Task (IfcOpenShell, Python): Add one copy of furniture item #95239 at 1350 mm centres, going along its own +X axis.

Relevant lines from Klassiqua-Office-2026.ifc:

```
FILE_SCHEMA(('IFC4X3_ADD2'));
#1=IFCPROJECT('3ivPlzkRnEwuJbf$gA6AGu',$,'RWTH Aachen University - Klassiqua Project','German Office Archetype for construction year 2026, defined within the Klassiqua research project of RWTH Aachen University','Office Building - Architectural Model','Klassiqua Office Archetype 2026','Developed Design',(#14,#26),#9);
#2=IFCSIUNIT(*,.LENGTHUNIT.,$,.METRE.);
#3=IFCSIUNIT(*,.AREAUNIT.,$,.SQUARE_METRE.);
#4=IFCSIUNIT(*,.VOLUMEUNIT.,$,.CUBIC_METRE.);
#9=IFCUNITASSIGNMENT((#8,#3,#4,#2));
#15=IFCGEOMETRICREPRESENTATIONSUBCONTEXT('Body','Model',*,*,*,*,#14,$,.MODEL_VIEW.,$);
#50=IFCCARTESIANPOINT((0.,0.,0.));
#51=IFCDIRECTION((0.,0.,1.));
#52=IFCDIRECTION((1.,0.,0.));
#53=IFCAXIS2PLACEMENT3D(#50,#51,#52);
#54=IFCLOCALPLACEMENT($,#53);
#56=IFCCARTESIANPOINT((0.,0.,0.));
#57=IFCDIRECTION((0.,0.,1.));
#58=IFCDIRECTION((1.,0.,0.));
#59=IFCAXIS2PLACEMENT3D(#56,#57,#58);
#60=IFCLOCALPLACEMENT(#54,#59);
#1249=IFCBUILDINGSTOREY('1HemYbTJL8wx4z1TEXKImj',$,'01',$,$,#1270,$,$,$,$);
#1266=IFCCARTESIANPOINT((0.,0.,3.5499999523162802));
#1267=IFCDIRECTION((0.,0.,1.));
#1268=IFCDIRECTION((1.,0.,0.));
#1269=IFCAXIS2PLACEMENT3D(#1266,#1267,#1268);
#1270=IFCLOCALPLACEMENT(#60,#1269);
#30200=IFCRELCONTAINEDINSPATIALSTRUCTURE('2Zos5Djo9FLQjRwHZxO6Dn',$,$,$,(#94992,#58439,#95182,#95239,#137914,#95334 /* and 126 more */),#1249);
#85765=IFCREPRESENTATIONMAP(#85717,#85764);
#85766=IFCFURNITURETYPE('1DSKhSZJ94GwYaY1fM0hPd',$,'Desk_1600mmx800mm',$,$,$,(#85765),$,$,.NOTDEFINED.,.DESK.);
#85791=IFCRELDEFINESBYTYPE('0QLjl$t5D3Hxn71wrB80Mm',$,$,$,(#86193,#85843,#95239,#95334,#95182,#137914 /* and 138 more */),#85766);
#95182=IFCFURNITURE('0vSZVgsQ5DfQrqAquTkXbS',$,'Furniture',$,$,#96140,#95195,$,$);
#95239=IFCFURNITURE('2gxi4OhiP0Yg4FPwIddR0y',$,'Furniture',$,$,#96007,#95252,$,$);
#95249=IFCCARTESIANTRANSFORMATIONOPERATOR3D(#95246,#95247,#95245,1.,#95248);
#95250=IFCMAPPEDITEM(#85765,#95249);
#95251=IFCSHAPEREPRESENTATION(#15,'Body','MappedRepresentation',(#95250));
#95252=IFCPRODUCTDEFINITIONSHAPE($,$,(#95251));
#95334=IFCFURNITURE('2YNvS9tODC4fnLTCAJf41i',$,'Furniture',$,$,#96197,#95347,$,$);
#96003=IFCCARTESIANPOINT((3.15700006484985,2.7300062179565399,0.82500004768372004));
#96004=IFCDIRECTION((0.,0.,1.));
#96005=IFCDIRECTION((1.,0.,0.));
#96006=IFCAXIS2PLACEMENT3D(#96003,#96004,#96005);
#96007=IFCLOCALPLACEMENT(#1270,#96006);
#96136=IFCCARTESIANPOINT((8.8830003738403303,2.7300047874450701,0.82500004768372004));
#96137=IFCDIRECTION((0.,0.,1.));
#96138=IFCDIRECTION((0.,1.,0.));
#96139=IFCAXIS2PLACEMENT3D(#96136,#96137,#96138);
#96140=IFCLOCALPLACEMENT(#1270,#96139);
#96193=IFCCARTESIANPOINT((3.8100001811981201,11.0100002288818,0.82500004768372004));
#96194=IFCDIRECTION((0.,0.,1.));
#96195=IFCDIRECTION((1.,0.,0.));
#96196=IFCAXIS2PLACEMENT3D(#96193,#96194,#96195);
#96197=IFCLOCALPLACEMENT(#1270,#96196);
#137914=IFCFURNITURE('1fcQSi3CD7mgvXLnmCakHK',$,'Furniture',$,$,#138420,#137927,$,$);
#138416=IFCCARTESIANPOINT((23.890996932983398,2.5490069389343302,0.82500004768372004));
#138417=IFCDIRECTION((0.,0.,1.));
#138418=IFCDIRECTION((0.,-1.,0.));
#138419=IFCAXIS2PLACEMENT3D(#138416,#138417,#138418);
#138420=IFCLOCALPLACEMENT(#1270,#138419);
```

```python
import ifcopenshell
import ifcopenshell.api.geometry
import ifcopenshell.api.root
import ifcopenshell.util.element
import ifcopenshell.util.placement

model = ifcopenshell.open("Klassiqua-Office-2026.ifc")

source = model.by_guid("2gxi4OhiP0Yg4FPwIddR0y")
base = ifcopenshell.util.placement.get_local_placement(source.ObjectPlacement)
step = base[:3, 0] * 1.35

for i in range(1, 2):
    copy = ifcopenshell.api.root.copy_class(model, product=source)
    copy.Representation = ifcopenshell.util.element.copy_deep(
        model, source.Representation, exclude=["IfcGeometricRepresentationContext", "IfcRepresentationMap"]
    )
    matrix = base.copy()
    matrix[:3, 3] += i * step
    print("added at", matrix[:3, 3].round(3) + 0.0)
    ifcopenshell.api.geometry.edit_object_placement(model, product=copy, matrix=matrix, is_si=False)

model.write("Klassiqua-Office-2026-out.ifc")
```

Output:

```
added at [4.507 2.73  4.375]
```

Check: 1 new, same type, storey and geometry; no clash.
